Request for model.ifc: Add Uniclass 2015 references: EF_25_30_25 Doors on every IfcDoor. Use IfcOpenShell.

First a look at what the model holds.

```python
import ifcopenshell

model = ifcopenshell.open("model.ifc")
print(model.schema)
print("classifications:", [c.Name for c in model.by_type("IfcClassification")])
for ifc_class in ("IfcDoor", "IfcRoof", "IfcStair", "IfcWall", "IfcWindow"):
    print(ifc_class, len(model.by_type(ifc_class)))
```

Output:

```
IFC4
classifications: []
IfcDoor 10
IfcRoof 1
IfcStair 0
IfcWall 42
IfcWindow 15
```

```python
import ifcopenshell
import ifcopenshell.api.classification

model = ifcopenshell.open("model.ifc")

system = ifcopenshell.api.classification.add_classification(model, classification="Uniclass 2015")

codes = {
    "IfcDoor": ("EF_25_30_25", "Doors"),
}
for ifc_class, (code, name) in codes.items():
    products = model.by_type(ifc_class)
    ifcopenshell.api.classification.add_reference(
        model, products=products, classification=system, identification=code, name=name
    )
    print(code, len(products))

model.write("model_v2.ifc")
```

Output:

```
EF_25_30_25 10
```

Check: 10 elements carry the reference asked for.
